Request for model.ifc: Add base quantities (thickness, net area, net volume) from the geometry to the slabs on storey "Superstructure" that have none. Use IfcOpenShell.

First a look at what the model holds.

```python
import ifcopenshell
import ifcopenshell.util.element
import ifcopenshell.util.unit

model = ifcopenshell.open("model.ifc")
print(model.schema)
for unit_type in ("LENGTHUNIT", "AREAUNIT", "VOLUMEUNIT"):
    print(unit_type, ifcopenshell.util.unit.calculate_unit_scale(model, unit_type))
storey = next(s for s in model.by_type("IfcBuildingStorey") if s.Name == "Superstructure")
slabs = [e for e in ifcopenshell.util.element.get_decomposition(storey) if e.is_a("IfcSlab")]
for e in sorted(slabs, key=lambda e: e.id()):
    print(e.id(), e.is_a(), e.Name, list(ifcopenshell.util.element.get_psets(e, qtos_only=True)), sep=" | ")
```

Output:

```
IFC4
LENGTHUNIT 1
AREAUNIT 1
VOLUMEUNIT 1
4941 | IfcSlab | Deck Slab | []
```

```python
import ifcopenshell
import ifcopenshell.api.pset
import ifcopenshell.geom
import ifcopenshell.util.element
import ifcopenshell.util.shape
import ifcopenshell.util.unit

model = ifcopenshell.open("model.ifc")
unit_scale = ifcopenshell.util.unit.calculate_unit_scale(model)
area_scale = ifcopenshell.util.unit.calculate_unit_scale(model, "AREAUNIT")
volume_scale = ifcopenshell.util.unit.calculate_unit_scale(model, "VOLUMEUNIT")
settings = ifcopenshell.geom.settings()

storey = next(s for s in model.by_type("IfcBuildingStorey") if s.Name == "Superstructure")
slabs = [e for e in ifcopenshell.util.element.get_decomposition(storey) if e.is_a("IfcSlab")]

for e in sorted(slabs, key=lambda e: e.id()):
    if ifcopenshell.util.element.get_psets(e, qtos_only=True, should_inherit=False):
        continue
    # Geometry comes back in metres, in the element's own axes.
    shape = ifcopenshell.geom.create_shape(settings, e)
    values = {
        "Width": ifcopenshell.util.shape.get_z(shape.geometry) / unit_scale,
        "NetArea": ifcopenshell.util.shape.get_footprint_area(shape.geometry) / area_scale,
        "NetVolume": ifcopenshell.util.shape.get_volume(shape.geometry) / volume_scale,
    }
    qto = ifcopenshell.api.pset.add_qto(model, product=e, name="Qto_SlabBaseQuantities")
    ifcopenshell.api.pset.edit_qto(model, qto=qto, properties=values)
    print(e.id(), {k: round(v, 3) for k, v in values.items()})

model.write("model-out.ifc")
```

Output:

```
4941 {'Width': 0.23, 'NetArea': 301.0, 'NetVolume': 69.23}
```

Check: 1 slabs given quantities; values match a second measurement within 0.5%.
